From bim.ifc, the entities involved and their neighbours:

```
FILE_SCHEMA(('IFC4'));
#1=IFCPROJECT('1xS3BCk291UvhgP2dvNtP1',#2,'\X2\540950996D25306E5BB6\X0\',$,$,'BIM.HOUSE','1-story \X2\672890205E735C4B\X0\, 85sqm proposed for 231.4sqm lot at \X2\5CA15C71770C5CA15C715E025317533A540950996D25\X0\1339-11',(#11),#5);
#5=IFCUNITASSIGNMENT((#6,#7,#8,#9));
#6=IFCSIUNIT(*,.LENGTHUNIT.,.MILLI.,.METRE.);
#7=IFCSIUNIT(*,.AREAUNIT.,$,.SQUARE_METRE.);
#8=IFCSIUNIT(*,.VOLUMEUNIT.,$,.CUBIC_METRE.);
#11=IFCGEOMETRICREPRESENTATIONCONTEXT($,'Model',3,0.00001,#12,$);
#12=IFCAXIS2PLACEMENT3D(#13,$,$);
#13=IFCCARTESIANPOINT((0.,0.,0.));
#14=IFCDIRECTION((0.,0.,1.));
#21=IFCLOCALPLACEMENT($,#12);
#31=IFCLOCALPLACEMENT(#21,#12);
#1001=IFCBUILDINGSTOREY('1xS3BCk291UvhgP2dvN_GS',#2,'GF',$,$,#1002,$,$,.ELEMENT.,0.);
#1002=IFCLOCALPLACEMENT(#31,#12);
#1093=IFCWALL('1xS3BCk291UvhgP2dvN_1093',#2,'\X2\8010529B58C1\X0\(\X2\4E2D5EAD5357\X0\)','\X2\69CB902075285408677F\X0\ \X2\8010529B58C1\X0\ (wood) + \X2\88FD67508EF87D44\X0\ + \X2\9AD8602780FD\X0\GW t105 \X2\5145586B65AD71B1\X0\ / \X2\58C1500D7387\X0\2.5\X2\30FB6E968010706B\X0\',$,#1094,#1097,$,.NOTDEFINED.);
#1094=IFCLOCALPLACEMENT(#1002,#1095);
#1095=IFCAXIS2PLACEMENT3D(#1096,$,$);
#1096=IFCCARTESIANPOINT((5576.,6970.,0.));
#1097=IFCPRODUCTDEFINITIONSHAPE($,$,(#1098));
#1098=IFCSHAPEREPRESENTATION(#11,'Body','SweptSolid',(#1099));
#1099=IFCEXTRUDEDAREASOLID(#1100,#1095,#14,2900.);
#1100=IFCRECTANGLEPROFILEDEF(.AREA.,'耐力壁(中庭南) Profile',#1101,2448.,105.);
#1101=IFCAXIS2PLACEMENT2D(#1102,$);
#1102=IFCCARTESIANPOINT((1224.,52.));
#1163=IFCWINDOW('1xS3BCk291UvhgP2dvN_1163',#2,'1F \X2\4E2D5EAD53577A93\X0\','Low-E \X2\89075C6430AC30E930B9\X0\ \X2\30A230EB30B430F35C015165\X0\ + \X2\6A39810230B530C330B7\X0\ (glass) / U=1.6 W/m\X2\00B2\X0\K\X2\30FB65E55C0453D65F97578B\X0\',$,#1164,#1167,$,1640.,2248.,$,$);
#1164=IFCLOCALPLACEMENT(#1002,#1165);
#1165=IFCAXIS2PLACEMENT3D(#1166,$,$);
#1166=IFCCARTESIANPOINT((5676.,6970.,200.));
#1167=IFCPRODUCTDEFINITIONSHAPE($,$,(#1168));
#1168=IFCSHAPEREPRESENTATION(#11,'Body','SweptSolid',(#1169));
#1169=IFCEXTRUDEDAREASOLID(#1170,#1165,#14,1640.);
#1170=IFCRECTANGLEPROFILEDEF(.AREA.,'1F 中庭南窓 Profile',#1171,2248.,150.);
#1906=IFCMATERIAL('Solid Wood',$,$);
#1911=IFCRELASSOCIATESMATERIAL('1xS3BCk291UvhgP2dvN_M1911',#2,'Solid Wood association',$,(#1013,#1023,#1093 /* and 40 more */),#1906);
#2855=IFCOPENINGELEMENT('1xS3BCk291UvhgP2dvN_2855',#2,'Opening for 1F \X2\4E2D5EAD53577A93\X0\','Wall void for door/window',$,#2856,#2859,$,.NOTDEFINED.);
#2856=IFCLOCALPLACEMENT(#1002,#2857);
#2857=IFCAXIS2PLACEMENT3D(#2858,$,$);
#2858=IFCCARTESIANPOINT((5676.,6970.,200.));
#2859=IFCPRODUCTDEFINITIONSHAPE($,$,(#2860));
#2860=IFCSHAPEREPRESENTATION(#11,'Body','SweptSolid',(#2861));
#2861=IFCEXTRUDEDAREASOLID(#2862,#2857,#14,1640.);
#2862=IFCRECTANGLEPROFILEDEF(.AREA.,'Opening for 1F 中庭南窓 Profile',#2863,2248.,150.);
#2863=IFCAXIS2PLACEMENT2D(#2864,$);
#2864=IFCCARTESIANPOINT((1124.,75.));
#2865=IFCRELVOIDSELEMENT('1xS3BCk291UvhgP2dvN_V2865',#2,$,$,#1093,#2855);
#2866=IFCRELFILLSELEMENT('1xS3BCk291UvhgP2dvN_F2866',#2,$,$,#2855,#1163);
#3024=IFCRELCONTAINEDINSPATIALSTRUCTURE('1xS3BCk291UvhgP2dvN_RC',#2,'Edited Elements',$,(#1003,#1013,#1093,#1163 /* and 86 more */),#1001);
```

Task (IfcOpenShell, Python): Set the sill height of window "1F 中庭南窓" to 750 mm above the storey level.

```python
import numpy as np
import ifcopenshell
import ifcopenshell.api.geometry
import ifcopenshell.geom
import ifcopenshell.util.element
import ifcopenshell.util.placement
import ifcopenshell.util.shape
import ifcopenshell.util.unit

model = ifcopenshell.open("bim.ifc")
unit_scale = ifcopenshell.util.unit.calculate_unit_scale(model)

window = model.by_guid("1xS3BCk291UvhgP2dvN_1163")
opening = window.FillsVoids[0].RelatingOpeningElement
storey = ifcopenshell.util.element.get_container(window, ifc_class="IfcBuildingStorey")
level = ifcopenshell.util.placement.get_local_placement(storey.ObjectPlacement)[2, 3]

# The opening's origin need not be at the sill, so measure its lowest point.
shape = ifcopenshell.geom.create_shape(ifcopenshell.geom.settings(), opening)
bottom = ifcopenshell.util.shape.get_shape_bottom_elevation(shape, shape.geometry) / unit_scale
dz = level + 0.75 / unit_scale - bottom

shift = np.array([0.0, 0.0, dz])
# The window is not placed relative to its opening, so move both.
for product in (opening, window):
    matrix = ifcopenshell.util.placement.get_local_placement(product.ObjectPlacement)
    matrix[:3, 3] += shift
    ifcopenshell.api.geometry.edit_object_placement(model, product=product, matrix=matrix, is_si=False)

print(f"moved by {dz * unit_scale:+.3f} m")

model.write("bim_edited.ifc")
```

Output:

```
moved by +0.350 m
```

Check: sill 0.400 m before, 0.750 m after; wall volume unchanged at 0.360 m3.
